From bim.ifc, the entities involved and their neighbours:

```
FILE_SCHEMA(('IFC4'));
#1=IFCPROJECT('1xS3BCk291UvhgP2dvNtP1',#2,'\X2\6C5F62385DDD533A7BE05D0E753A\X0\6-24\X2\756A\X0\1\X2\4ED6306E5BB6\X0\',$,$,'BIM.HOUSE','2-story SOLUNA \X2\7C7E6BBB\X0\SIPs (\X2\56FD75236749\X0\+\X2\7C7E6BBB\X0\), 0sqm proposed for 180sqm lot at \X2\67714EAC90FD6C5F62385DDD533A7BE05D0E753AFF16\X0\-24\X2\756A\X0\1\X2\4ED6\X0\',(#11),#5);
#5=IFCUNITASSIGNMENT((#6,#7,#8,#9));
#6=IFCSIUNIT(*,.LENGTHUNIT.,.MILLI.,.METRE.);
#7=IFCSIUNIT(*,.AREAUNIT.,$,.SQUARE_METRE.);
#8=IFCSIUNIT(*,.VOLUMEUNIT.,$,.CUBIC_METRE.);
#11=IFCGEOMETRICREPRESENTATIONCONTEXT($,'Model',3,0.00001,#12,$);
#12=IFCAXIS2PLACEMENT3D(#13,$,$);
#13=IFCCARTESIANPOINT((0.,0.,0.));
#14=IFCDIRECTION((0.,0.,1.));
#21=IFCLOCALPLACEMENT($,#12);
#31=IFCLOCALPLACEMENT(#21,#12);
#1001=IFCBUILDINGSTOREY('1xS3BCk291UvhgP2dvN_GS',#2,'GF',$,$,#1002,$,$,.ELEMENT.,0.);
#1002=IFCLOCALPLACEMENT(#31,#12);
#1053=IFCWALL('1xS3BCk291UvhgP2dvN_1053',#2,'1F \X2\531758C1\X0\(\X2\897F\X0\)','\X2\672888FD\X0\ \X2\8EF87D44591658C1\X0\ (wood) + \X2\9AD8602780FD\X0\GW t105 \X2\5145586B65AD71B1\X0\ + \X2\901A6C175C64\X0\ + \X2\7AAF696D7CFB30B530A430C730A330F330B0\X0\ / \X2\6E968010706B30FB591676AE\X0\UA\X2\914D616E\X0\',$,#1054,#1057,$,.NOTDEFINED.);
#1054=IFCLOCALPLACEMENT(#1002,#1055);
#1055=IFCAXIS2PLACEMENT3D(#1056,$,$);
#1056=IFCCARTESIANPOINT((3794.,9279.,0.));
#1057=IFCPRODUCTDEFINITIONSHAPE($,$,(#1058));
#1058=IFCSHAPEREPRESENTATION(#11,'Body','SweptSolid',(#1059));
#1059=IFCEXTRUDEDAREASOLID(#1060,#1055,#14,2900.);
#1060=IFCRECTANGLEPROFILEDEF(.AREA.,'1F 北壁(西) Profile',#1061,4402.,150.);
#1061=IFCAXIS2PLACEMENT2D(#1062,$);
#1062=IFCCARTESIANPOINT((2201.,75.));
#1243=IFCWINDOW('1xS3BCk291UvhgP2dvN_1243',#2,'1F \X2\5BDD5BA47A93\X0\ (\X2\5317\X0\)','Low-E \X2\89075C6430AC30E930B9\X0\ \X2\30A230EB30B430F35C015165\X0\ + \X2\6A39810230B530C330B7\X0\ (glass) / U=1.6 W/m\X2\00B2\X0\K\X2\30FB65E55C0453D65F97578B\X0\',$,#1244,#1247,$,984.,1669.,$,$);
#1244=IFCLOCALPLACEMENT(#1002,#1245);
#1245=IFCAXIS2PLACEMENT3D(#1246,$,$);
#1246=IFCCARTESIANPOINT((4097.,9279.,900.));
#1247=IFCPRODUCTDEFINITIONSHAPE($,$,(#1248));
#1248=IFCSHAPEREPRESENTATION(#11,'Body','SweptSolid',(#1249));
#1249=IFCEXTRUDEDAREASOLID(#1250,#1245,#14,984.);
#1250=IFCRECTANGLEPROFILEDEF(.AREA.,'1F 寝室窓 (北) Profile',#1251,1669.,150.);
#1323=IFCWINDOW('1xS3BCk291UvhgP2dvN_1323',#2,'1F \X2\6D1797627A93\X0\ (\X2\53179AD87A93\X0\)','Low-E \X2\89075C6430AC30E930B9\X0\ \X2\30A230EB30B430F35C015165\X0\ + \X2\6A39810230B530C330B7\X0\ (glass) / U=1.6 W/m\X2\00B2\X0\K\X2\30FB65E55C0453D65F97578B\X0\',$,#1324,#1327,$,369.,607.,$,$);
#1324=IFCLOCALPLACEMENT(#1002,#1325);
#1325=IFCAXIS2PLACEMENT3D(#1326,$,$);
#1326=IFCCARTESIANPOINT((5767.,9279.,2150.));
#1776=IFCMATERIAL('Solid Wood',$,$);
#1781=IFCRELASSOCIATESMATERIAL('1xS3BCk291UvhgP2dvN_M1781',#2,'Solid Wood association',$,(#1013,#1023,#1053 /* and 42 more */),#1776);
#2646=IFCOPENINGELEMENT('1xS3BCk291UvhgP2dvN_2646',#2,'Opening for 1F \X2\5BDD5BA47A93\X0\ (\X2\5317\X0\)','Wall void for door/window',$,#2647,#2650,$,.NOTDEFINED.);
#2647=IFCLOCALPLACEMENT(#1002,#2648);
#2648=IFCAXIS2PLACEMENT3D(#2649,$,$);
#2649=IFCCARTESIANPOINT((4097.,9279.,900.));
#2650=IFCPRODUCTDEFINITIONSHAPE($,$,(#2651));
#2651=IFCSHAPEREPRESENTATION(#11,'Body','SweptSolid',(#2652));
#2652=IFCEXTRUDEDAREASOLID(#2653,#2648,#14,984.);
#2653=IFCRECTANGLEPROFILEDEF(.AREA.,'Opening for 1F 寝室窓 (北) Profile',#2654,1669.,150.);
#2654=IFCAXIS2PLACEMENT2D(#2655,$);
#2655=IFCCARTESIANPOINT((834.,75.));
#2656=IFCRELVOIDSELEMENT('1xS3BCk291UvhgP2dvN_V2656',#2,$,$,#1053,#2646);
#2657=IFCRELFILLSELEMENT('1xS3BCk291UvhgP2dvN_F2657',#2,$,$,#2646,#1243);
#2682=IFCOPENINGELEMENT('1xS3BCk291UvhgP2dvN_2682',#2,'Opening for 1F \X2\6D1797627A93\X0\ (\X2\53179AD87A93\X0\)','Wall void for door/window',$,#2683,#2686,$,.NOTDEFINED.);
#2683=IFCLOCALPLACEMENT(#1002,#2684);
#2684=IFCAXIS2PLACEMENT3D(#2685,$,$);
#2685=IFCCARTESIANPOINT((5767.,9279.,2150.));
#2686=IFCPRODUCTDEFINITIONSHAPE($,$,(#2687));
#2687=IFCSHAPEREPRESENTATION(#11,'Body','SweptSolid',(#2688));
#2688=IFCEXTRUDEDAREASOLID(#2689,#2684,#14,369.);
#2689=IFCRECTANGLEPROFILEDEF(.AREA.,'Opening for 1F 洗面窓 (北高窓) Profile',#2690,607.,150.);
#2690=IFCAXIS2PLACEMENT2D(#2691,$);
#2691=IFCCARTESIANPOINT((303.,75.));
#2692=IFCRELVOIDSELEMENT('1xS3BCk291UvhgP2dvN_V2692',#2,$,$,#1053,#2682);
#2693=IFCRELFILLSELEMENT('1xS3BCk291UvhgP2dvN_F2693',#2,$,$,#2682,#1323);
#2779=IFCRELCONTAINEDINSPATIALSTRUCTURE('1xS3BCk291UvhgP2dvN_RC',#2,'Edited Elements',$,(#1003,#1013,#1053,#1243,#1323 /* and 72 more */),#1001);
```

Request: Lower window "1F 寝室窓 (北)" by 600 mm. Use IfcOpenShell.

```python
import numpy as np
import ifcopenshell
import ifcopenshell.api.geometry
import ifcopenshell.util.placement
import ifcopenshell.util.unit

model = ifcopenshell.open("bim.ifc")
unit_scale = ifcopenshell.util.unit.calculate_unit_scale(model)

window = model.by_id(1243)
opening = window.FillsVoids[0].RelatingOpeningElement
dz = -0.6 / unit_scale

shift = np.array([0.0, 0.0, dz])
# The window is not placed relative to its opening, so move both.
for product in (opening, window):
    matrix = ifcopenshell.util.placement.get_local_placement(product.ObjectPlacement)
    matrix[:3, 3] += shift
    ifcopenshell.api.geometry.edit_object_placement(model, product=product, matrix=matrix, is_si=False)

print(f"moved by {dz * unit_scale:+.3f} m")

model.write("bim-out.ifc")
```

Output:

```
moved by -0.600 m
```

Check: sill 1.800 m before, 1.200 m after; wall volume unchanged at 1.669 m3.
